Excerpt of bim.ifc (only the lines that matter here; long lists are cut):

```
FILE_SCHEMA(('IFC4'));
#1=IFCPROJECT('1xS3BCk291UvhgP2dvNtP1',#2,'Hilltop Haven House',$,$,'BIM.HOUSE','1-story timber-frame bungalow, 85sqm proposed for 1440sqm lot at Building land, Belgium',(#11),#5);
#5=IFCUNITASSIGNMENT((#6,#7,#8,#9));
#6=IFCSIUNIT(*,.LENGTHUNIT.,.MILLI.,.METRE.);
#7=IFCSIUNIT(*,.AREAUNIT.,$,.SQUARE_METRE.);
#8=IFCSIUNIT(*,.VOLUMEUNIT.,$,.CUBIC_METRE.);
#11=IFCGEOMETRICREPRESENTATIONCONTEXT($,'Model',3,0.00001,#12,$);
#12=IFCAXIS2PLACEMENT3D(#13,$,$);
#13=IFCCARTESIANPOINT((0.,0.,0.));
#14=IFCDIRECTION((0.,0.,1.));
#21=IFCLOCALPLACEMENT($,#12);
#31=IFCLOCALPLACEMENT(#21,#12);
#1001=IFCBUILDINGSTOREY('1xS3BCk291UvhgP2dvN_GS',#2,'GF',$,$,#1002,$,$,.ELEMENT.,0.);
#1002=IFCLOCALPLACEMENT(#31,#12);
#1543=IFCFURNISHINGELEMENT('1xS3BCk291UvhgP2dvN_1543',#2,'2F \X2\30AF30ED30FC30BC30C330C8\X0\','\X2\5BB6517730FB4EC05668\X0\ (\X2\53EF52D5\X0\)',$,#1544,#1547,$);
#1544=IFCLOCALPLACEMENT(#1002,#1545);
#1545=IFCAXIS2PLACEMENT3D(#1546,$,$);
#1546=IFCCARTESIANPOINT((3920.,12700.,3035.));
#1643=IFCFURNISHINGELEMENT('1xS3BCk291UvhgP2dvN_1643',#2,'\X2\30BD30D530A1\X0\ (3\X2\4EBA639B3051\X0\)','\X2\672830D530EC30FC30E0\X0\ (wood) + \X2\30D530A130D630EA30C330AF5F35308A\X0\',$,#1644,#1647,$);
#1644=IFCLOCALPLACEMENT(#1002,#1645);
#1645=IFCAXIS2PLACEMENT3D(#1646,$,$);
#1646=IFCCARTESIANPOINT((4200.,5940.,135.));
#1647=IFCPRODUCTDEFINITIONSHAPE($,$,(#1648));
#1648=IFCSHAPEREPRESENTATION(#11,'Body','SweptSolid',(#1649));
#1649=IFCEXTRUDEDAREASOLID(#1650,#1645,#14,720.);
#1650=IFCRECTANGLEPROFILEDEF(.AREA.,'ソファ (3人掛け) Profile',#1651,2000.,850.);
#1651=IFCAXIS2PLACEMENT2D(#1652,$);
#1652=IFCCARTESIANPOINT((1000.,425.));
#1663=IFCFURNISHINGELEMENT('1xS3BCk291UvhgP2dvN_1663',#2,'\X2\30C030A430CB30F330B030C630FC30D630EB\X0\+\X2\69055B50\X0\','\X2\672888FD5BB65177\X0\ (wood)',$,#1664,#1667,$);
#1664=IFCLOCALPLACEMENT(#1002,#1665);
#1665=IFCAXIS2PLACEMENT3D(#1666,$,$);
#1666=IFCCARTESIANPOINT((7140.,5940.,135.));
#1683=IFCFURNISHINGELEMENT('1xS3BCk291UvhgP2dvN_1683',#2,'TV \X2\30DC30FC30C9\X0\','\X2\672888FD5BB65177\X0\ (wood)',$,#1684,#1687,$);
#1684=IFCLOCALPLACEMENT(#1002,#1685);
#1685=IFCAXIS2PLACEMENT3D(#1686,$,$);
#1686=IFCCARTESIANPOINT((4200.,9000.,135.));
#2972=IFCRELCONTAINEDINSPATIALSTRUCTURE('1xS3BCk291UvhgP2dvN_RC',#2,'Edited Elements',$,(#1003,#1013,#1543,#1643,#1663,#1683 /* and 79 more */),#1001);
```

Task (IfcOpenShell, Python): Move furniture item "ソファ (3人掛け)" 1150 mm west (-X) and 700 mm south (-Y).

```python
import ifcopenshell
import ifcopenshell.api.geometry
import ifcopenshell.util.placement

model = ifcopenshell.open("bim.ifc")

item = model.by_id(1643)
matrix = ifcopenshell.util.placement.get_local_placement(item.ObjectPlacement)
matrix[0, 3] -= 1150.0
matrix[1, 3] -= 700.0
ifcopenshell.api.geometry.edit_object_placement(model, product=item, matrix=matrix, is_si=False)

print(ifcopenshell.util.placement.get_local_placement(item.ObjectPlacement).round(3) + 0.0)

model.write("bim_edited.ifc")
```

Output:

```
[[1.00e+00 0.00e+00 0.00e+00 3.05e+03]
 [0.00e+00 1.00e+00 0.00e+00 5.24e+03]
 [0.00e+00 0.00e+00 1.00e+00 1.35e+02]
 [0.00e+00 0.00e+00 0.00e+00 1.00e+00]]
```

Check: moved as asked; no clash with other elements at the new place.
